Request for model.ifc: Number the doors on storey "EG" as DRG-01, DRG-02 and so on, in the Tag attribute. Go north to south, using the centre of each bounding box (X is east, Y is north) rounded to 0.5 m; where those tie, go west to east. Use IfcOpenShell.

First a look at what the model holds.

```python
import ifcopenshell
import ifcopenshell.util.element
import ifcopenshell.util.placement

model = ifcopenshell.open("model.ifc")
print(model.schema)
storey = next(s for s in model.by_type("IfcBuildingStorey") if s.Name == "EG")
doors = [e for e in ifcopenshell.util.element.get_decomposition(storey) if e.is_a("IfcDoor")]
for e in sorted(doors, key=lambda e: e.id()):
    origin = ifcopenshell.util.placement.get_local_placement(e.ObjectPlacement)[:3, 3]
    print(e.id(), e.Tag, e.Name, origin.round(2) + 0.0, sep=" | ")
```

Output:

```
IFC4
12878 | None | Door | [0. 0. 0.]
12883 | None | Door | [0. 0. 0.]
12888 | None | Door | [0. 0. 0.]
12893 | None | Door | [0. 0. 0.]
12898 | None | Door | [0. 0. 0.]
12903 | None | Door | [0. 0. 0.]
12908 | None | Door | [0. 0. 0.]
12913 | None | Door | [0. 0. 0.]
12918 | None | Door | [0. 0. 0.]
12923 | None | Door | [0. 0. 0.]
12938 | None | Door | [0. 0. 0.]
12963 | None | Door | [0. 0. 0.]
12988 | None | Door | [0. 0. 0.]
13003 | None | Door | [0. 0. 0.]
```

```python
import ifcopenshell
import ifcopenshell.geom
import ifcopenshell.util.element
import ifcopenshell.util.shape

model = ifcopenshell.open("model.ifc")
settings = ifcopenshell.geom.settings()
settings.set("use-world-coords", True)


def centre(element):
    shape = ifcopenshell.geom.create_shape(settings, element)
    return ifcopenshell.util.shape.get_bbox_centroid(shape.geometry)


storey = next(s for s in model.by_type("IfcBuildingStorey") if s.Name == "EG")
doors = [e for e in ifcopenshell.util.element.get_decomposition(storey) if e.is_a("IfcDoor")]

# Insertion points can sit at a corner or the storey origin, so sort by the geometry (in metres).
centres = {e: centre(e) for e in doors}
doors.sort(key=lambda e: (-round(centres[e][1] / 0.5), centres[e][0]))

for i, e in enumerate(doors, start=1):
    number = f"DRG-{i:02d}"
    e.Tag = number
    print(e.id(), number)

model.write("model_edited.ifc")
```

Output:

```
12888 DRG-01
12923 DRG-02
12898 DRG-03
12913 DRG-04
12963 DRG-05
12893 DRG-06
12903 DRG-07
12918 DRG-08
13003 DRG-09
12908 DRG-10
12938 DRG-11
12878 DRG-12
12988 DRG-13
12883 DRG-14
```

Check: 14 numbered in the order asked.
